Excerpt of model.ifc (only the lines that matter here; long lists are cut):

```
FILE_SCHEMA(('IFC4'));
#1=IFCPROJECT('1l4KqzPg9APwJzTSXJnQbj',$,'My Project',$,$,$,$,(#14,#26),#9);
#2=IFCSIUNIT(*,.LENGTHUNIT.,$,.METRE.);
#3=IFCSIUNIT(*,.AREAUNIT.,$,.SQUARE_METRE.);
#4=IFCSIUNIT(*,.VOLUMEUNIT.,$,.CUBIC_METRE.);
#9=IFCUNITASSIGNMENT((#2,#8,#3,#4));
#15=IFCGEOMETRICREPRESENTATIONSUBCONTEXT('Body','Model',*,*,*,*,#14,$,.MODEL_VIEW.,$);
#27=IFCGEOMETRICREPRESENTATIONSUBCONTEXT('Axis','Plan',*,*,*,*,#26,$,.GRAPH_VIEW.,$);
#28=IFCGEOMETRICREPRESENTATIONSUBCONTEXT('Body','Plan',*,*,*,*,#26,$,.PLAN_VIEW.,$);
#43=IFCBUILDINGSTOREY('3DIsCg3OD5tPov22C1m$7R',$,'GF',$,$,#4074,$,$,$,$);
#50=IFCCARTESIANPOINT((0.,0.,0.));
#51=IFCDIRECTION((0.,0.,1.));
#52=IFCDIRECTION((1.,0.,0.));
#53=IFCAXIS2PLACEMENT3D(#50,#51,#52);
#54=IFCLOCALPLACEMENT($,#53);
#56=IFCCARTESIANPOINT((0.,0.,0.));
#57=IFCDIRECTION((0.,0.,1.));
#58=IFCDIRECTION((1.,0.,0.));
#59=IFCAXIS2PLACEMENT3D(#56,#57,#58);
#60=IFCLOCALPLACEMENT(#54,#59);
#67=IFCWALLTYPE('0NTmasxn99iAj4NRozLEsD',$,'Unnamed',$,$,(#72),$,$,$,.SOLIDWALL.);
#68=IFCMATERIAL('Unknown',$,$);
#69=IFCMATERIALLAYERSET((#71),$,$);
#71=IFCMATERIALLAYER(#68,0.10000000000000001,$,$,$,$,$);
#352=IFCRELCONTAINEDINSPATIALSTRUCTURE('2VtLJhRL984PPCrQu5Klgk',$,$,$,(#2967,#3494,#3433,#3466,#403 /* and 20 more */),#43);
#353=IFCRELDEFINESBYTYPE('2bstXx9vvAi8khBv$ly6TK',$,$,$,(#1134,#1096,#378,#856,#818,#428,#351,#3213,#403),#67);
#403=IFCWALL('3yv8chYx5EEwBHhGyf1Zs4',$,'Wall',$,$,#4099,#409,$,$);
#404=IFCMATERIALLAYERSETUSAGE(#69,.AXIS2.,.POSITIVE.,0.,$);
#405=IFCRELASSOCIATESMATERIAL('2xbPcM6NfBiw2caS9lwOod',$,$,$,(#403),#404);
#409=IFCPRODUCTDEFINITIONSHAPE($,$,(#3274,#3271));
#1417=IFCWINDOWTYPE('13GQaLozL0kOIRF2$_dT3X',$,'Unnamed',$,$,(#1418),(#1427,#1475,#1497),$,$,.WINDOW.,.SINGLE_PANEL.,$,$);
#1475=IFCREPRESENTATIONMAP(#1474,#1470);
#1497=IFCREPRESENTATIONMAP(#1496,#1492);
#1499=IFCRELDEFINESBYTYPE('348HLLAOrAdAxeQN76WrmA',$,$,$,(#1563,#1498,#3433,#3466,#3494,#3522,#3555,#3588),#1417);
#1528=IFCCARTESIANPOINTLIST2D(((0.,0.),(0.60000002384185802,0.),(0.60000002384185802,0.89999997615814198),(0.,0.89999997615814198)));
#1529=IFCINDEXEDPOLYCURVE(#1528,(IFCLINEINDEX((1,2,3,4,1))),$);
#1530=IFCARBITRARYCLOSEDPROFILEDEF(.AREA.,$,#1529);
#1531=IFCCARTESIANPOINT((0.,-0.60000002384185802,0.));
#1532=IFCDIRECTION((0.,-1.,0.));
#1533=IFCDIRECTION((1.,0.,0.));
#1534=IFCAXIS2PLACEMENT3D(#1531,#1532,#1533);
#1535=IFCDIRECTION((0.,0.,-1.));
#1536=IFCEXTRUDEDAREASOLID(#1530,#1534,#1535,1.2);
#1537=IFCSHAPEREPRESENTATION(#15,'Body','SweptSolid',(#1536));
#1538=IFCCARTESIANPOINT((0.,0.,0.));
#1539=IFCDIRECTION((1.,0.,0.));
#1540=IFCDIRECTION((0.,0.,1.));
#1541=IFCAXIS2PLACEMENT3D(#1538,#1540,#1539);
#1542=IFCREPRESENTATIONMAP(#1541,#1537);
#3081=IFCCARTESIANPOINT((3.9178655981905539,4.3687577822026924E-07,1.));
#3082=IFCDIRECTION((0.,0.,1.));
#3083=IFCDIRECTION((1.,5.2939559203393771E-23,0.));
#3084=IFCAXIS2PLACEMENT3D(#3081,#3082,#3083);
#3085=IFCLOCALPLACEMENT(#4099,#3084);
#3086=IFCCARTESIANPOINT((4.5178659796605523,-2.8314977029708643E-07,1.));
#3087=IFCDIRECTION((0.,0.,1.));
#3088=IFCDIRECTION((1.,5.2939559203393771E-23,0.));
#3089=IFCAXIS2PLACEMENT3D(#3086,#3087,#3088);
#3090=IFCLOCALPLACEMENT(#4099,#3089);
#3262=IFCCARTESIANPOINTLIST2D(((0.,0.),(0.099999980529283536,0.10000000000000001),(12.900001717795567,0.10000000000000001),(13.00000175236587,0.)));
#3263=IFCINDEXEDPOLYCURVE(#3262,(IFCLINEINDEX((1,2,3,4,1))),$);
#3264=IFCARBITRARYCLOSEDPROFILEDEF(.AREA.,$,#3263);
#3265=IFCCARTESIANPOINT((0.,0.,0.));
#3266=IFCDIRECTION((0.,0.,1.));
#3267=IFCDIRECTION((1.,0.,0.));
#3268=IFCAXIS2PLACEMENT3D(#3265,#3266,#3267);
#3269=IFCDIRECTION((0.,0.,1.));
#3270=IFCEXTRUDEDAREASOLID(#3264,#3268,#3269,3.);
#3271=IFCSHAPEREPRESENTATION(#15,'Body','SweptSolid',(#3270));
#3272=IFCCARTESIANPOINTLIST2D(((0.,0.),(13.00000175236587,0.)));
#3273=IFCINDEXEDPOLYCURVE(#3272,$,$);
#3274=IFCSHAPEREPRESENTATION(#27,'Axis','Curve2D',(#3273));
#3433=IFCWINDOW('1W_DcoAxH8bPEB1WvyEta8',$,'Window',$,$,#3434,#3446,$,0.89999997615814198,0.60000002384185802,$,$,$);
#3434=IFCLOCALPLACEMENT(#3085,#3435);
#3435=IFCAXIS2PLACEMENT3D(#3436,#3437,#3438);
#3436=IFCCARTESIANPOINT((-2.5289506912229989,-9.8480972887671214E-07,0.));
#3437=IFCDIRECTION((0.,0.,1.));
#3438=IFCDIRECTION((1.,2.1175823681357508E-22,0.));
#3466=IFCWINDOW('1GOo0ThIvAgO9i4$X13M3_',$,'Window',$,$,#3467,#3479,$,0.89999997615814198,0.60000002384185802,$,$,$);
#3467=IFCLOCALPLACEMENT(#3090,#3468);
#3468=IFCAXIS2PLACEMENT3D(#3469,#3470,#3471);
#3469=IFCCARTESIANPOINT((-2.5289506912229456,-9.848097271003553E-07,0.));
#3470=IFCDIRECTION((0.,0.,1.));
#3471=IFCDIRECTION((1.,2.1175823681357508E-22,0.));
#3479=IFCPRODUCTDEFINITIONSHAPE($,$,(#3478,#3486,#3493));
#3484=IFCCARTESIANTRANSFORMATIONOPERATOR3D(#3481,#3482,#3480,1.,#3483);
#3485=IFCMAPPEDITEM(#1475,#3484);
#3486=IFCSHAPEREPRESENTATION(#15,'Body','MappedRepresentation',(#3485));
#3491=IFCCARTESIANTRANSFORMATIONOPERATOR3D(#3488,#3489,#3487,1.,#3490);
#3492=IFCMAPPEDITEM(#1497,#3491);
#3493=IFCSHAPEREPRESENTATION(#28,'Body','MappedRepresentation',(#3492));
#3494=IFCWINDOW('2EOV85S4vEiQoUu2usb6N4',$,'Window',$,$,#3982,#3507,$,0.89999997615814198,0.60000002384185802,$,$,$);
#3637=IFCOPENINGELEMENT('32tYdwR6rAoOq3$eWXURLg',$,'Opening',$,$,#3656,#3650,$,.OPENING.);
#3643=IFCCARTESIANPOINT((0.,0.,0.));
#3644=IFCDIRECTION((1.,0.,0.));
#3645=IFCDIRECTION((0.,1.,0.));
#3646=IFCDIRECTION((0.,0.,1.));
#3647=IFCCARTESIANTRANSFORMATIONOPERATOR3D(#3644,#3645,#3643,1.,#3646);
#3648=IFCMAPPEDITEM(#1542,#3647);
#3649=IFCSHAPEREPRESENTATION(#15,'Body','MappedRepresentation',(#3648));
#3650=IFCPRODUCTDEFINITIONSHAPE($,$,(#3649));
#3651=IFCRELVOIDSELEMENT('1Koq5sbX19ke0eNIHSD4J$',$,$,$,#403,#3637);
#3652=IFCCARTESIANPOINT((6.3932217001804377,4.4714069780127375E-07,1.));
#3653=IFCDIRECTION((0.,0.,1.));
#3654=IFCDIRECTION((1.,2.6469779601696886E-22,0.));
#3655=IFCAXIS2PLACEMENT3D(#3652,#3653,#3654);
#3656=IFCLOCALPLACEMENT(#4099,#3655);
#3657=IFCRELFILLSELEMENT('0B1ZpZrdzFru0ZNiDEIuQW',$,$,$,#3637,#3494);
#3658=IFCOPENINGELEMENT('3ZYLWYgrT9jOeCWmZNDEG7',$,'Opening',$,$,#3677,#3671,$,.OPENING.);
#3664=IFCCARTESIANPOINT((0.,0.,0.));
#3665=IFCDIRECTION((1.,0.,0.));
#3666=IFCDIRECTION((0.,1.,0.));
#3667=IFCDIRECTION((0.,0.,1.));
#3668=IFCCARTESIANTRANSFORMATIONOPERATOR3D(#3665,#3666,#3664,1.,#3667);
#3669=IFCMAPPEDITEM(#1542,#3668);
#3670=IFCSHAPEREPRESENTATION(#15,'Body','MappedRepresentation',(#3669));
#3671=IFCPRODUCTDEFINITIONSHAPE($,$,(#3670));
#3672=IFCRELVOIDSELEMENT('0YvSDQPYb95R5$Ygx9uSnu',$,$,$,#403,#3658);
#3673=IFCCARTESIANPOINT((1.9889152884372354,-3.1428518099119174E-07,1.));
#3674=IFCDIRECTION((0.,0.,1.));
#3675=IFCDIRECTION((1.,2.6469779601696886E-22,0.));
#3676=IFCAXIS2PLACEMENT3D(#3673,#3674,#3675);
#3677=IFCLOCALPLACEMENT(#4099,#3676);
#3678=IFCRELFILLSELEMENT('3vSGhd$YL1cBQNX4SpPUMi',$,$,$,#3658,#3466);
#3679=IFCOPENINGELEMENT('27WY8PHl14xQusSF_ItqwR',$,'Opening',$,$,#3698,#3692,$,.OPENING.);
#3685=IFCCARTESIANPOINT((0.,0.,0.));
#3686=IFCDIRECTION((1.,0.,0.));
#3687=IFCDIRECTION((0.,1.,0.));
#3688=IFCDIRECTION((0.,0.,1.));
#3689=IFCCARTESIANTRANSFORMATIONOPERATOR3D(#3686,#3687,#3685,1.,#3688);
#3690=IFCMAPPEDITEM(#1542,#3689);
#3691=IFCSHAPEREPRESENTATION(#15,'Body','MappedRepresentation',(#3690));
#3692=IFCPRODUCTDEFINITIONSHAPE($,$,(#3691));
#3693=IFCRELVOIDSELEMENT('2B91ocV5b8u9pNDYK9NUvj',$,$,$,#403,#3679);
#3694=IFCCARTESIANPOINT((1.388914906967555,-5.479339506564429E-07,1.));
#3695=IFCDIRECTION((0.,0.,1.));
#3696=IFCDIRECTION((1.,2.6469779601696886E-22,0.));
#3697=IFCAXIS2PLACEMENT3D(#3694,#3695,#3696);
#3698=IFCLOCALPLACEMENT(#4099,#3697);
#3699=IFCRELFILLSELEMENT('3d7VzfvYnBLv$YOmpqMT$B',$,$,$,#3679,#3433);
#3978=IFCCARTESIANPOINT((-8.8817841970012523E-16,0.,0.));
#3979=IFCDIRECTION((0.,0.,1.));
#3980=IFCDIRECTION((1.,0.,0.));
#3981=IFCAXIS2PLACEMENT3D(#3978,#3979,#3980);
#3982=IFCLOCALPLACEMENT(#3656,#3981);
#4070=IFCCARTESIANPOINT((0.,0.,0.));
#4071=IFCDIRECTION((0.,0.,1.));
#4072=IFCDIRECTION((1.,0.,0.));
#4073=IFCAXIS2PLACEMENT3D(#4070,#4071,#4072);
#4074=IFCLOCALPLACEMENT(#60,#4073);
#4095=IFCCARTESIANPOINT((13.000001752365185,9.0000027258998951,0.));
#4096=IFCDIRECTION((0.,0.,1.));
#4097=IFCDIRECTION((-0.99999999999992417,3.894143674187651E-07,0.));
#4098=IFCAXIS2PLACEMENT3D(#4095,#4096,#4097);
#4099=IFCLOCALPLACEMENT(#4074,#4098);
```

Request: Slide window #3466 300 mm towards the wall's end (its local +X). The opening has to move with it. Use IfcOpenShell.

```python
import ifcopenshell
import ifcopenshell.api.geometry
import ifcopenshell.util.placement

model = ifcopenshell.open("model.ifc")

window = model.by_id(3466)
opening = window.FillsVoids[0].RelatingOpeningElement
wall = opening.VoidsElements[0].RelatingBuildingElement

wall_matrix = ifcopenshell.util.placement.get_local_placement(wall.ObjectPlacement)
shift = wall_matrix[:3, 0] * 0.3
before = ifcopenshell.util.placement.get_local_placement(window.ObjectPlacement)[:3, 3].copy()

# The window is not placed relative to its opening, so move both.
for product in (opening, window):
    matrix = ifcopenshell.util.placement.get_local_placement(product.ObjectPlacement)
    matrix[:3, 3] += shift
    ifcopenshell.api.geometry.edit_object_placement(model, product=product, matrix=matrix, is_si=False)

after = ifcopenshell.util.placement.get_local_placement(window.ObjectPlacement)[:3, 3]
print("window moved by", (after - before).round(3) + 0.0)

model.write("model_edited.ifc")
```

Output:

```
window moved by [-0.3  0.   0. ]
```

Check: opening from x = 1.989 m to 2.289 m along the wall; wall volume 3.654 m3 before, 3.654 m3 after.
